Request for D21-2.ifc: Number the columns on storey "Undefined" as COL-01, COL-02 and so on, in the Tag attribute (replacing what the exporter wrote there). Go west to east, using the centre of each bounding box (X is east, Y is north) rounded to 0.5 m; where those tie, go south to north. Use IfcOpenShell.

First a look at what the model holds.

```python
import ifcopenshell
import ifcopenshell.util.element
import ifcopenshell.util.placement

model = ifcopenshell.open("D21-2.ifc")
print(model.schema)
storey = next(s for s in model.by_type("IfcBuildingStorey") if s.Name == "Undefined")
columns = [e for e in ifcopenshell.util.element.get_decomposition(storey) if e.is_a("IfcColumn")]
for e in sorted(columns, key=lambda e: e.id()):
    origin = ifcopenshell.util.placement.get_local_placement(e.ObjectPlacement)[:3, 3]
    print(e.id(), e.Tag, e.Name, origin.round(2) + 0.0, sep=" | ")
```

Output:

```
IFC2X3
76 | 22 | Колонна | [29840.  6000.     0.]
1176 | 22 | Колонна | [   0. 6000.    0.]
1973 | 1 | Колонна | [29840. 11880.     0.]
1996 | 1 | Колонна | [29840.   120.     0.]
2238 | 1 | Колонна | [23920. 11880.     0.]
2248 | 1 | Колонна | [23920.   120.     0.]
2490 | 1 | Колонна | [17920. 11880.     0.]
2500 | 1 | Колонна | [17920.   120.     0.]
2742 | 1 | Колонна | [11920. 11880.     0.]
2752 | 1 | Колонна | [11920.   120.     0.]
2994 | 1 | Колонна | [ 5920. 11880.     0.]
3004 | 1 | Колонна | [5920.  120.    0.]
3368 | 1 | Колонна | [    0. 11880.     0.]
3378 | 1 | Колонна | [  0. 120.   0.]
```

```python
import ifcopenshell
import ifcopenshell.geom
import ifcopenshell.util.element
import ifcopenshell.util.shape

model = ifcopenshell.open("D21-2.ifc")
settings = ifcopenshell.geom.settings()
settings.set("use-world-coords", True)


def centre(element):
    shape = ifcopenshell.geom.create_shape(settings, element)
    return ifcopenshell.util.shape.get_bbox_centroid(shape.geometry)


storey = next(s for s in model.by_type("IfcBuildingStorey") if s.Name == "Undefined")
columns = [e for e in ifcopenshell.util.element.get_decomposition(storey) if e.is_a("IfcColumn")]

# Insertion points can sit at a corner or the storey origin, so sort by the geometry (in metres).
centres = {e: centre(e) for e in columns}
columns.sort(key=lambda e: (round(centres[e][0] / 0.5), centres[e][1]))

for i, e in enumerate(columns, start=1):
    number = f"COL-{i:02d}"
    e.Tag = number
    print(e.id(), number)

model.write("D21-2_rev.ifc")
```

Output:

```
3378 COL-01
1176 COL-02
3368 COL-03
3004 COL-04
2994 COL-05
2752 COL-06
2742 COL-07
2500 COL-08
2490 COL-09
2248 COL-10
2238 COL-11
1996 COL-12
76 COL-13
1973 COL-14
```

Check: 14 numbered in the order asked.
